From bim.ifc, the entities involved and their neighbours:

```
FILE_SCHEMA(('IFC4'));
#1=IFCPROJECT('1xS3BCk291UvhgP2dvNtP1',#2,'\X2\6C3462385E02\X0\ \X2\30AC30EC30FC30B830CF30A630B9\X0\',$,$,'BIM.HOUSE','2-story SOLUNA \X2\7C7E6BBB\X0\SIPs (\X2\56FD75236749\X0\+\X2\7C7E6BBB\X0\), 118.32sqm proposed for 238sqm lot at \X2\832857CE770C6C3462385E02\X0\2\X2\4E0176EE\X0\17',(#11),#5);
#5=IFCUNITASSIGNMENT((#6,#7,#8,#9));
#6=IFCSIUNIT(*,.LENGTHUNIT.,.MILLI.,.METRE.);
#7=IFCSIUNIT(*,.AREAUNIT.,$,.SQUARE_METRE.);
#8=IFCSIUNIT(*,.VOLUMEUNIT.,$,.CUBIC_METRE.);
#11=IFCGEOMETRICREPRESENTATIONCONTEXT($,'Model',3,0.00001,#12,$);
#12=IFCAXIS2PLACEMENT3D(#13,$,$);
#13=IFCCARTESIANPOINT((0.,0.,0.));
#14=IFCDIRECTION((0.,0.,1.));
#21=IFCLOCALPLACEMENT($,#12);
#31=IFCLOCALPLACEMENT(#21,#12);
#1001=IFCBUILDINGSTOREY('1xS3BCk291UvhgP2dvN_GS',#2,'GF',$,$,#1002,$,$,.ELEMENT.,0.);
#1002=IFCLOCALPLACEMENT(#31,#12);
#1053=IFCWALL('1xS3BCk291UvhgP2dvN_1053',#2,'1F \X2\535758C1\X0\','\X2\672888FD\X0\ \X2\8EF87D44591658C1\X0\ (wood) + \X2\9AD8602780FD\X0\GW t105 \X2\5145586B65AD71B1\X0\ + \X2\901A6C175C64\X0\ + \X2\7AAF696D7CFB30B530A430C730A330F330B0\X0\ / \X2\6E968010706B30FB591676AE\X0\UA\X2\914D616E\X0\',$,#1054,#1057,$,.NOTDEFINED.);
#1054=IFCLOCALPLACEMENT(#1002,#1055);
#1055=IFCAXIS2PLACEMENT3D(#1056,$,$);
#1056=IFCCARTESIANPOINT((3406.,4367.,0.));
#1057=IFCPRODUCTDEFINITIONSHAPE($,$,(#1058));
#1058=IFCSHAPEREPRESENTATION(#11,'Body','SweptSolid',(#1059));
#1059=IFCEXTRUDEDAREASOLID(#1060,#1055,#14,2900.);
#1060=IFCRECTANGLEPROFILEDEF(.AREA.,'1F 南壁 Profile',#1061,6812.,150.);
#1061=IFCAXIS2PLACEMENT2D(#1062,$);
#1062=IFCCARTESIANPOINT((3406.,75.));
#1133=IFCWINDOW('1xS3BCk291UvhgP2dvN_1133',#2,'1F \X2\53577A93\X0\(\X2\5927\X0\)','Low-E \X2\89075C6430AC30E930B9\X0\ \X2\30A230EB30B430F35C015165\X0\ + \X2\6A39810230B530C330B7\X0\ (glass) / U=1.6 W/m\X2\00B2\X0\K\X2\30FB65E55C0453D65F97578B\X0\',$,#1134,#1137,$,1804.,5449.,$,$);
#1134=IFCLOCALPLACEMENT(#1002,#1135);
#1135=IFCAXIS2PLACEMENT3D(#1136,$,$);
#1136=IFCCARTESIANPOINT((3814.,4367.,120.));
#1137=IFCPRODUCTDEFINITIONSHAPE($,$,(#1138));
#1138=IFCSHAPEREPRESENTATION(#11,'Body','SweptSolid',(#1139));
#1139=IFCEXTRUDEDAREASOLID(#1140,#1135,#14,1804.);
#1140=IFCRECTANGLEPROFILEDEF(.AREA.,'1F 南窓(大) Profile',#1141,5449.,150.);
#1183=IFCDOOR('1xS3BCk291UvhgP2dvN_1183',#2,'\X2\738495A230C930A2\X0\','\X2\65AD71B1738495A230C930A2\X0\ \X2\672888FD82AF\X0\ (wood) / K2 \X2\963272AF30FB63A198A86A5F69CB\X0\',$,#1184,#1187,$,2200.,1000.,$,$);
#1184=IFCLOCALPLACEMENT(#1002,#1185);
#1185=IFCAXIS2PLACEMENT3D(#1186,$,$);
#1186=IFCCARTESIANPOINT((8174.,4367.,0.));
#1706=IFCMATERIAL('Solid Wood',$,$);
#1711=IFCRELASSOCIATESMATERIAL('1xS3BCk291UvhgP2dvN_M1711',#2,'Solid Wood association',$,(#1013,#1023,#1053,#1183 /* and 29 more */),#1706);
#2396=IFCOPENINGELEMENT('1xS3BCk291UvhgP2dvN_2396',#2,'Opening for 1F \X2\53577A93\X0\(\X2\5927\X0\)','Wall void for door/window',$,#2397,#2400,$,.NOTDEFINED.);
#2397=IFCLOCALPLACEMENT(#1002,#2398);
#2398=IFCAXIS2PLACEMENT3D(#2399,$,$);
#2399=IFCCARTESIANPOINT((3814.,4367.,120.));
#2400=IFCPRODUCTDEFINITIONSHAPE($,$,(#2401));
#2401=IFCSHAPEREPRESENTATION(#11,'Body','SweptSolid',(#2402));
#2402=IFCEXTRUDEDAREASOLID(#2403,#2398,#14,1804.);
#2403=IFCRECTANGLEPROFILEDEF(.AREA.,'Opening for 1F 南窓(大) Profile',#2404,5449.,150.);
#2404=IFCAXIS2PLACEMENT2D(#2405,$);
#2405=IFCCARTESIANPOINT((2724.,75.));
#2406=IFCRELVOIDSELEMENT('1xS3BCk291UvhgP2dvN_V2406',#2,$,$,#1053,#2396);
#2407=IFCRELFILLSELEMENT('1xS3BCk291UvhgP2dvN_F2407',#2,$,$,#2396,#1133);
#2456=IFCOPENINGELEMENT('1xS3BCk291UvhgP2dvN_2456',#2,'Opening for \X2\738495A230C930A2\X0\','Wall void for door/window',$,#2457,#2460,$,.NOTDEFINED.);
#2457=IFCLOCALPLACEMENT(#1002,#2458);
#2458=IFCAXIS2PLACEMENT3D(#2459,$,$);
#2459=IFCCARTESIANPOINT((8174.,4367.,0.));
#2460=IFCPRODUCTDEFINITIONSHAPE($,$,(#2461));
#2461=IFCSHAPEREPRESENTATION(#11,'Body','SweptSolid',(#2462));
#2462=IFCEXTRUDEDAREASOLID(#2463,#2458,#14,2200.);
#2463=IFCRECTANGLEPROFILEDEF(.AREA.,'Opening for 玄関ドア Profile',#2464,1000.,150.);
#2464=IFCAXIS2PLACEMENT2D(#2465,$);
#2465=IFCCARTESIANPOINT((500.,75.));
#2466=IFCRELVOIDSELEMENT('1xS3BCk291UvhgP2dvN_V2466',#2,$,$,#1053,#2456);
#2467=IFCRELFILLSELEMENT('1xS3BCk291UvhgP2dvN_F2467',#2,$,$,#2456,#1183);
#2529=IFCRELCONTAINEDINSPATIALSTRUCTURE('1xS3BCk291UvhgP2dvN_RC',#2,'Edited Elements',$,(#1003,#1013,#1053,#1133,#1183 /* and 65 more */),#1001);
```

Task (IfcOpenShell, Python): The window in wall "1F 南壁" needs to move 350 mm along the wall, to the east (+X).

```python
import ifcopenshell
import ifcopenshell.api.geometry
import ifcopenshell.util.placement

model = ifcopenshell.open("bim.ifc")

window = model.by_id(1133)
opening = window.FillsVoids[0].RelatingOpeningElement
wall = opening.VoidsElements[0].RelatingBuildingElement

wall_matrix = ifcopenshell.util.placement.get_local_placement(wall.ObjectPlacement)
shift = wall_matrix[:3, 0] * 350.0
before = ifcopenshell.util.placement.get_local_placement(window.ObjectPlacement)[:3, 3].copy()

# The window is not placed relative to its opening, so move both.
for product in (opening, window):
    matrix = ifcopenshell.util.placement.get_local_placement(product.ObjectPlacement)
    matrix[:3, 3] += shift
    ifcopenshell.api.geometry.edit_object_placement(model, product=product, matrix=matrix, is_si=False)

after = ifcopenshell.util.placement.get_local_placement(window.ObjectPlacement)[:3, 3]
print("window moved by", (after - before).round(3) + 0.0)

model.write("bim_edited.ifc")
```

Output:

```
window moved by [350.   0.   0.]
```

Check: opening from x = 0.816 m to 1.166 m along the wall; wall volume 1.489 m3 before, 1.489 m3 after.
